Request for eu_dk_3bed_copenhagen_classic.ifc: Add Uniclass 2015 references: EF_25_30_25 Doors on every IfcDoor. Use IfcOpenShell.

First a look at what the model holds.

```python
import ifcopenshell

model = ifcopenshell.open("eu_dk_3bed_copenhagen_classic.ifc")
print(model.schema)
print("classifications:", [c.Name for c in model.by_type("IfcClassification")])
for ifc_class in ("IfcDoor", "IfcRoof", "IfcStair", "IfcWall", "IfcWindow"):
    print(ifc_class, len(model.by_type(ifc_class)))
```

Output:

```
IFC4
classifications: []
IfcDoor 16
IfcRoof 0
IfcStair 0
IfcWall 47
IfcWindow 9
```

```python
import ifcopenshell
import ifcopenshell.api.classification

model = ifcopenshell.open("eu_dk_3bed_copenhagen_classic.ifc")

system = ifcopenshell.api.classification.add_classification(model, classification="Uniclass 2015")

codes = {
    "IfcDoor": ("EF_25_30_25", "Doors"),
}
for ifc_class, (code, name) in codes.items():
    products = model.by_type(ifc_class)
    ifcopenshell.api.classification.add_reference(
        model, products=products, classification=system, identification=code, name=name
    )
    print(code, len(products))

model.write("eu_dk_3bed_copenhagen_classic_edited.ifc")
```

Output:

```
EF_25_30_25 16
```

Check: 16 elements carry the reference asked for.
